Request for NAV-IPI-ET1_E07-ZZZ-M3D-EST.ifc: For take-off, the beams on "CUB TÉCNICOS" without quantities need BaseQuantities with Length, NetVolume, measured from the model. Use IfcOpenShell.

First a look at what the model holds.

```python
import ifcopenshell
import ifcopenshell.util.element
import ifcopenshell.util.unit

model = ifcopenshell.open("NAV-IPI-ET1_E07-ZZZ-M3D-EST.ifc")
print(model.schema)
for unit_type in ("LENGTHUNIT", "AREAUNIT", "VOLUMEUNIT"):
    print(unit_type, ifcopenshell.util.unit.calculate_unit_scale(model, unit_type))
storey = next(s for s in model.by_type("IfcBuildingStorey") if s.Name == "CUB TÉCNICOS")
beams = [e for e in ifcopenshell.util.element.get_decomposition(storey) if e.is_a("IfcBeam")]
for e in sorted(beams, key=lambda e: e.id()):
    print(e.id(), e.is_a(), e.Name, list(ifcopenshell.util.element.get_psets(e, qtos_only=True)), sep=" | ")
```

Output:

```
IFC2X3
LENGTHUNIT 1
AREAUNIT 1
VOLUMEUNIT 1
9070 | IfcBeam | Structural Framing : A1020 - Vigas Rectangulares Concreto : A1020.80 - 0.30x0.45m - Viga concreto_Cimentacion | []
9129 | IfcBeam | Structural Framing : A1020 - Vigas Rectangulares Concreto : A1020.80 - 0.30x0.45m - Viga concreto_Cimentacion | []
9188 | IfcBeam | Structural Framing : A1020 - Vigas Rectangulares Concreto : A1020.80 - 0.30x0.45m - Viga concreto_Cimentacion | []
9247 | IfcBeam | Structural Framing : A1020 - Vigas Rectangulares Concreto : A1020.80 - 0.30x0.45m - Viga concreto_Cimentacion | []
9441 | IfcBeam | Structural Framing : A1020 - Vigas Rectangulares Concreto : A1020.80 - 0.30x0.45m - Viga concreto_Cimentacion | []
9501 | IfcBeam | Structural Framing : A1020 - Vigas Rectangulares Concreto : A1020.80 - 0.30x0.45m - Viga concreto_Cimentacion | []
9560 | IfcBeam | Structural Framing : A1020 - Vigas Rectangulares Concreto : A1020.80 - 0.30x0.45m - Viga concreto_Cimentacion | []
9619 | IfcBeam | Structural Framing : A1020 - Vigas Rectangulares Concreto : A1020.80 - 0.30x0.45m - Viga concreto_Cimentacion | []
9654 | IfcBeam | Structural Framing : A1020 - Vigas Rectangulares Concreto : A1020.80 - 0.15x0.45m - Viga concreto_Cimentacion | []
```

```python
import ifcopenshell
import ifcopenshell.api.pset
import ifcopenshell.geom
import ifcopenshell.util.element
import ifcopenshell.util.shape
import ifcopenshell.util.unit

model = ifcopenshell.open("NAV-IPI-ET1_E07-ZZZ-M3D-EST.ifc")
unit_scale = ifcopenshell.util.unit.calculate_unit_scale(model)
volume_scale = ifcopenshell.util.unit.calculate_unit_scale(model, "VOLUMEUNIT")
settings = ifcopenshell.geom.settings()

storey = next(s for s in model.by_type("IfcBuildingStorey") if s.Name == "CUB TÉCNICOS")
beams = [e for e in ifcopenshell.util.element.get_decomposition(storey) if e.is_a("IfcBeam")]

for e in sorted(beams, key=lambda e: e.id()):
    if ifcopenshell.util.element.get_psets(e, qtos_only=True, should_inherit=False):
        continue
    # Geometry comes back in metres, in the element's own axes.
    shape = ifcopenshell.geom.create_shape(settings, e)
    values = {
        "Length": ifcopenshell.util.shape.get_max_xyz(shape.geometry) / unit_scale,
        "NetVolume": ifcopenshell.util.shape.get_volume(shape.geometry) / volume_scale,
    }
    qto = ifcopenshell.api.pset.add_qto(model, product=e, name="BaseQuantities")
    ifcopenshell.api.pset.edit_qto(model, qto=qto, properties=values)
    print(e.id(), {k: round(v, 3) for k, v in values.items()})

model.write("NAV-IPI-ET1_E07-ZZZ-M3D-EST_rev.ifc")
```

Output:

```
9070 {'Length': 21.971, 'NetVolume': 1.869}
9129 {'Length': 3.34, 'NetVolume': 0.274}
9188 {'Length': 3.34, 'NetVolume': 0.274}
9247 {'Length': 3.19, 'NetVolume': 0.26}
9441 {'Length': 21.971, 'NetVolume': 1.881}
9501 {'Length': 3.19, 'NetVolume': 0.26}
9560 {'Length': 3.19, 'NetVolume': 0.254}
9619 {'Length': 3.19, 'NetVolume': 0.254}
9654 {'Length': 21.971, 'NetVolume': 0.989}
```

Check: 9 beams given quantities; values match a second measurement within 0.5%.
